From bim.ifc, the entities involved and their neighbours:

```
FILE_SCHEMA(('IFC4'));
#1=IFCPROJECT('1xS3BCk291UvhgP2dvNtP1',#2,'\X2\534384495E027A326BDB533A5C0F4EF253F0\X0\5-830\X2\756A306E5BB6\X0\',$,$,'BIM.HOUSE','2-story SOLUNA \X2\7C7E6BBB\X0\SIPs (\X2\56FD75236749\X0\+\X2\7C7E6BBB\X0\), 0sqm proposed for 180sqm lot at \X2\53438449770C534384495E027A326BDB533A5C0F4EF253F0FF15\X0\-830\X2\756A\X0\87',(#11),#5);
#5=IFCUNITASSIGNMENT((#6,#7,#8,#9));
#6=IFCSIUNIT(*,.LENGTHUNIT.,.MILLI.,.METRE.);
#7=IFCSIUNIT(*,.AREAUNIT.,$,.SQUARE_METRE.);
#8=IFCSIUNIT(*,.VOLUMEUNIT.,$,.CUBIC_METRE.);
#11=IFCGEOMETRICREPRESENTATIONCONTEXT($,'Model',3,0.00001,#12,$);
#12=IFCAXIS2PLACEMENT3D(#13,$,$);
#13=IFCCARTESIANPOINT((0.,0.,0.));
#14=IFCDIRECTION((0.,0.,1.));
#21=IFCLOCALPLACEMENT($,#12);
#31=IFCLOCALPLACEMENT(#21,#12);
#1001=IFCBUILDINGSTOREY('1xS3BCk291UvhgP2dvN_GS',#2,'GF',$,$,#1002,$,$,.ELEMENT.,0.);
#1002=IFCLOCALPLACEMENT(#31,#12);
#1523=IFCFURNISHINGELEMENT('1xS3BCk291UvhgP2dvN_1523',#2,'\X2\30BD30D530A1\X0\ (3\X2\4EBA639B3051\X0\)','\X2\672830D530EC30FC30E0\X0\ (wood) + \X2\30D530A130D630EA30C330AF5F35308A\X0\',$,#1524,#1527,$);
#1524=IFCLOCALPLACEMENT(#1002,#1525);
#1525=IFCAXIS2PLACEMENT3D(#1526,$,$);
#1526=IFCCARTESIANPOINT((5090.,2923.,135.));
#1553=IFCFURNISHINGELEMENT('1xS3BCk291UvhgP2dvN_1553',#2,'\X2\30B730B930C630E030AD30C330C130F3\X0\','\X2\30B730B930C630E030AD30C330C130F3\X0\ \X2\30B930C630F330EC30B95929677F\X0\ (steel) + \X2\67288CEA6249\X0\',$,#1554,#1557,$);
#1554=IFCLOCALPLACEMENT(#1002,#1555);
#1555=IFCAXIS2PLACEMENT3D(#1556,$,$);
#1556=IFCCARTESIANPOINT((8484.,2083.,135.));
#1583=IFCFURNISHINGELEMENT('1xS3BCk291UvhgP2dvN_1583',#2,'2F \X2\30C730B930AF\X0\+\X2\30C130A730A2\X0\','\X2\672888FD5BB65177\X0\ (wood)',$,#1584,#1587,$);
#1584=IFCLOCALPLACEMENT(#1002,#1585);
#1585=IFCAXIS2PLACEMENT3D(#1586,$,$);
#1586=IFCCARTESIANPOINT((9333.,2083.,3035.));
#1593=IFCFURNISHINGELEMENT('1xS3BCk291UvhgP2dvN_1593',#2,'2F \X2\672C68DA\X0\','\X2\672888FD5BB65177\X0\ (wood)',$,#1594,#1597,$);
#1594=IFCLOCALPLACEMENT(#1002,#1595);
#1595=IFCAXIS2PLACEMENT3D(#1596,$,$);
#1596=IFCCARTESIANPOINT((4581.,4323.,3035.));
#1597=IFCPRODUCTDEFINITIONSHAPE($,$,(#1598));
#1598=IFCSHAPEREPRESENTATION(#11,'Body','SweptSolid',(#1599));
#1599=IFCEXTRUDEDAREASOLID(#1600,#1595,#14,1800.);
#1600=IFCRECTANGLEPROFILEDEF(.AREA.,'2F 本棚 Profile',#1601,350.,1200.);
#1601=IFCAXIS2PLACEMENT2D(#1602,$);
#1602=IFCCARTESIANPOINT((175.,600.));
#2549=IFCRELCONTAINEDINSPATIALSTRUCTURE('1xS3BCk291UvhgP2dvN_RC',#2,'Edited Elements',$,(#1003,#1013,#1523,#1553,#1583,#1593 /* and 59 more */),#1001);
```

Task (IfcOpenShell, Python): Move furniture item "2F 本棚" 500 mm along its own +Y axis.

```python
import ifcopenshell
import ifcopenshell.api.geometry
import ifcopenshell.util.placement
import ifcopenshell.util.unit

model = ifcopenshell.open("bim.ifc")
unit_scale = ifcopenshell.util.unit.calculate_unit_scale(model)

item = model.by_guid("1xS3BCk291UvhgP2dvN_1593")
matrix = ifcopenshell.util.placement.get_local_placement(item.ObjectPlacement)
matrix[:3, 3] += matrix[:3, 1] * 0.5 / unit_scale
ifcopenshell.api.geometry.edit_object_placement(model, product=item, matrix=matrix, is_si=False)

print(ifcopenshell.util.placement.get_local_placement(item.ObjectPlacement).round(3) + 0.0)

model.write("bim_edited.ifc")
```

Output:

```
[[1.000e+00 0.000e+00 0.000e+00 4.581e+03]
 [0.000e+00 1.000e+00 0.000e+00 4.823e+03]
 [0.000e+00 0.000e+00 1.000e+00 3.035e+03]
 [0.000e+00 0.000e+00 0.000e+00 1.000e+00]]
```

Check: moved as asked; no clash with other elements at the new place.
